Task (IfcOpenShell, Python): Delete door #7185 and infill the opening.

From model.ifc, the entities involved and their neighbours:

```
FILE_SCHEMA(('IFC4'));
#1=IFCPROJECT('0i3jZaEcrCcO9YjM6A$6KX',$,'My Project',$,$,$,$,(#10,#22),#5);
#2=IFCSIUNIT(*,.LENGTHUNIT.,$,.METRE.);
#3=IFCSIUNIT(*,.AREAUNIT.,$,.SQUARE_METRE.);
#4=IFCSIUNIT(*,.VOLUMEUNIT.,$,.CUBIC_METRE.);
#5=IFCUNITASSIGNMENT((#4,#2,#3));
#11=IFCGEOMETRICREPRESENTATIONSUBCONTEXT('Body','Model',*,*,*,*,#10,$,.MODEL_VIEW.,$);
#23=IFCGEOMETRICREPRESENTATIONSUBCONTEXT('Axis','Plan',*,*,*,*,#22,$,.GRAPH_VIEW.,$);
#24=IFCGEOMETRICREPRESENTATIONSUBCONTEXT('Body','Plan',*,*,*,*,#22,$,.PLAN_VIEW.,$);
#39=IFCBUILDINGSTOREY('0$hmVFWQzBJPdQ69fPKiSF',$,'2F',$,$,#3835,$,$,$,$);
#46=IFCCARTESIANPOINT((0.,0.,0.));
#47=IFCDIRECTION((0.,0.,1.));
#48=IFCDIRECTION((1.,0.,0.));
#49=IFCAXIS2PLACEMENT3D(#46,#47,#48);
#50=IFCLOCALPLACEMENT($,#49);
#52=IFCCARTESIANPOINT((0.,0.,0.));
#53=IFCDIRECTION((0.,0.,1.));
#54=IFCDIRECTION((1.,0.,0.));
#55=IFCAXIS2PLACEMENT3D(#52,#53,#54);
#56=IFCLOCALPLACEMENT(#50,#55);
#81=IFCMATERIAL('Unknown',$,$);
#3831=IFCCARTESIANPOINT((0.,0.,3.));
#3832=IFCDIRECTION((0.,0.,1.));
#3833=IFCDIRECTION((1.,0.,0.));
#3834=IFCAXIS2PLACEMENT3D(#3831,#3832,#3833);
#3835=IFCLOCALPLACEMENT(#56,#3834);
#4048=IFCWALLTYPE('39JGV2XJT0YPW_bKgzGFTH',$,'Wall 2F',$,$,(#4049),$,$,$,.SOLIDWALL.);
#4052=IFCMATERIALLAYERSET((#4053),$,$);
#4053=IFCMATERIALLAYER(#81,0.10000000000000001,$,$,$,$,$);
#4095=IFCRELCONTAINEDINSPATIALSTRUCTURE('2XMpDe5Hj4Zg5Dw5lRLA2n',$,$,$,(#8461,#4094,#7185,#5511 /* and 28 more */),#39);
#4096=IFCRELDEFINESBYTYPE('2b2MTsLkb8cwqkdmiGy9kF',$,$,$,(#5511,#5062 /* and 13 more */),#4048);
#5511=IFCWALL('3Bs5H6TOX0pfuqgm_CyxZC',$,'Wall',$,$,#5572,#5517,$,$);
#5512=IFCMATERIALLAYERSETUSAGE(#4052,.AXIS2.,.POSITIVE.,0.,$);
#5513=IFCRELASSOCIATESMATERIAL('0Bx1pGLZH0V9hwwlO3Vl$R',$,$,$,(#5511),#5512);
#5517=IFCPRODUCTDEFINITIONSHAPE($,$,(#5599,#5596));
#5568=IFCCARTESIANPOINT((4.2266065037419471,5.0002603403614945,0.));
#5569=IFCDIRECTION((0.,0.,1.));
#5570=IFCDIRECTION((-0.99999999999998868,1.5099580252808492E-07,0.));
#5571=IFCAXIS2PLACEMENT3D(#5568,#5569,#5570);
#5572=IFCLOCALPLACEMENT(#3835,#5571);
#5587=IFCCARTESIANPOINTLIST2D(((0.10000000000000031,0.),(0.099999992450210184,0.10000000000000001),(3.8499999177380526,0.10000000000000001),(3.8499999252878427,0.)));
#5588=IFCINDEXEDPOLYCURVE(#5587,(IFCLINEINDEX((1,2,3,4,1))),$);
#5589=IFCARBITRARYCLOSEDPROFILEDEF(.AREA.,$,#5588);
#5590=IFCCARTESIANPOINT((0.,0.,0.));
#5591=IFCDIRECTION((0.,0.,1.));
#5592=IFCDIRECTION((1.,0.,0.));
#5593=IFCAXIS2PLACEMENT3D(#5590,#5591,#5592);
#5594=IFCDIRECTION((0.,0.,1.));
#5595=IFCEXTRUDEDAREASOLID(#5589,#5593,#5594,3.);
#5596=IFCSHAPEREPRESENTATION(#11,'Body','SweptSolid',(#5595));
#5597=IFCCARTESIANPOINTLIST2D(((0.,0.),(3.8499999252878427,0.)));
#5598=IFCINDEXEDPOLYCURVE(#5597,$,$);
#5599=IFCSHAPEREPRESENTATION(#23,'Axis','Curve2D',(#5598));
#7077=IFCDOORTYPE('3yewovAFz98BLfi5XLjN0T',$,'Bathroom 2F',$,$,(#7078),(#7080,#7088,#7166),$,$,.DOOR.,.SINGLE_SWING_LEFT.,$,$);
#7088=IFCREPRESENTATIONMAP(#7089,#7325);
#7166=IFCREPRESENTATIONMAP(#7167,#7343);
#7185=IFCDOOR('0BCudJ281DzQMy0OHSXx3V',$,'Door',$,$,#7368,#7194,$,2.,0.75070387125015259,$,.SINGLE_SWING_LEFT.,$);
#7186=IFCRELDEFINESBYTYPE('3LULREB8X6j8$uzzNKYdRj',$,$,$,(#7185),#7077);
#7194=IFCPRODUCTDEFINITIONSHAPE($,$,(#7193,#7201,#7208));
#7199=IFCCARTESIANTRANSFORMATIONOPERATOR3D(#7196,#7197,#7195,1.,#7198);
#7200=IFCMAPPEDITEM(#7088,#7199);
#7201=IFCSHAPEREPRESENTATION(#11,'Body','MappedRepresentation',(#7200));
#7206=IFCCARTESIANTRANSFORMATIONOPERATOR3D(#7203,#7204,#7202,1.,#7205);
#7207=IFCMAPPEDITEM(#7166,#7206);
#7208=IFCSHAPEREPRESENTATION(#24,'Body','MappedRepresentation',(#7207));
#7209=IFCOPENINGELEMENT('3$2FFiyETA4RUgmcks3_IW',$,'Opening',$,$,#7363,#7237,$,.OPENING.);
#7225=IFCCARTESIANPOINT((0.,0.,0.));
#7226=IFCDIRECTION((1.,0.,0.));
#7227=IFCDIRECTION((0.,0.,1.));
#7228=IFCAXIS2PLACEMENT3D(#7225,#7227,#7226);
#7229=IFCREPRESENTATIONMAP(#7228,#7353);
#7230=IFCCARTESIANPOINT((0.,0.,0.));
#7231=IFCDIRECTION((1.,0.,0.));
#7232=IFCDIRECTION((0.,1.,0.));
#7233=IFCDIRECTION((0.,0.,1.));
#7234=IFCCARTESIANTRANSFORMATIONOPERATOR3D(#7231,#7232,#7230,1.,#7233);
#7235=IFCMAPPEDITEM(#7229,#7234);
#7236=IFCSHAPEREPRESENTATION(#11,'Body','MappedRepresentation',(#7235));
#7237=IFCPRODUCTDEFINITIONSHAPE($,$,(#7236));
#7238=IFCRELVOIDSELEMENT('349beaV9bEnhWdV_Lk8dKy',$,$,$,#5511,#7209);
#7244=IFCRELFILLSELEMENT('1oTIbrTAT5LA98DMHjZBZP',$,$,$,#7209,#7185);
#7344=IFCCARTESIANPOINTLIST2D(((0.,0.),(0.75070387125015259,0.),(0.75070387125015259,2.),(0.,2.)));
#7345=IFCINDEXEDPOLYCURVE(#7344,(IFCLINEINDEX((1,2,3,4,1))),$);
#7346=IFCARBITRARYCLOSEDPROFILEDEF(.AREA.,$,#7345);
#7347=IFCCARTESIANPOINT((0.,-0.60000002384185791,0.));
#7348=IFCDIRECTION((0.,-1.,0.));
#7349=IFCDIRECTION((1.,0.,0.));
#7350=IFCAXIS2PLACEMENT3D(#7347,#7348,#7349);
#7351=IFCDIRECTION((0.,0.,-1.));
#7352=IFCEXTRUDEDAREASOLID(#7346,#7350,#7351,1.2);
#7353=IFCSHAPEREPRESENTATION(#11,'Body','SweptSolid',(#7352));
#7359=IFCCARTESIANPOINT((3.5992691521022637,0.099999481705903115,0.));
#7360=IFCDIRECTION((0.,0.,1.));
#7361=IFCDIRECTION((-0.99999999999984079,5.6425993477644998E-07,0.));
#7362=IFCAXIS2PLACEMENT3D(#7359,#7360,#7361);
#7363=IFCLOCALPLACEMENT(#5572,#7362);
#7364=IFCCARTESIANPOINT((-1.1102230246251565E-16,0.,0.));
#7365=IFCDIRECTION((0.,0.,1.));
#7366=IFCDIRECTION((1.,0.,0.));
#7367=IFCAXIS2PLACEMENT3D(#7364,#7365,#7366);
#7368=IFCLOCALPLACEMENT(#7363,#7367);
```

```python
import ifcopenshell
import ifcopenshell.api.feature
import ifcopenshell.api.root
import ifcopenshell.geom
import ifcopenshell.util.shape

model = ifcopenshell.open("model.ifc")
settings = ifcopenshell.geom.settings()


def volume(element):
    """Net volume in cubic metres, openings subtracted."""
    shape = ifcopenshell.geom.create_shape(settings, element)
    return ifcopenshell.util.shape.get_volume(shape.geometry)


door = model.by_id(7185)
opening = door.FillsVoids[0].RelatingOpeningElement
wall = opening.VoidsElements[0].RelatingBuildingElement
before = volume(wall)

ifcopenshell.api.root.remove_product(model, product=door)
ifcopenshell.api.feature.remove_feature(model, feature=opening)

after = volume(wall)

print(f"wall volume {before:.3f} -> {after:.3f} m3")

model.write("model_updated.ifc")
```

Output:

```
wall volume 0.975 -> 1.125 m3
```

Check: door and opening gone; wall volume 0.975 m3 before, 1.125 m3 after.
